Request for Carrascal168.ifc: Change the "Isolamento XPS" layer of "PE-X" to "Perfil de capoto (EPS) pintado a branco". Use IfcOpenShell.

First a look at what the model holds.

```python
import ifcopenshell
import ifcopenshell.util.element

model = ifcopenshell.open("Carrascal168.ifc")
print(model.schema)
for layer_set in model.by_type("IfcMaterialLayerSet"):
    if layer_set.LayerSetName == "PE-X":
        for layer in layer_set.MaterialLayers:
            print(layer.id(), layer.Material and layer.Material.Name, layer.LayerThickness, sep=" | ")
        print(len(ifcopenshell.util.element.get_elements_by_material(model, layer_set)), "elements and types use it")
print(sorted(m.Name for m in model.by_type("IfcMaterial") if m.Name)[:60])
```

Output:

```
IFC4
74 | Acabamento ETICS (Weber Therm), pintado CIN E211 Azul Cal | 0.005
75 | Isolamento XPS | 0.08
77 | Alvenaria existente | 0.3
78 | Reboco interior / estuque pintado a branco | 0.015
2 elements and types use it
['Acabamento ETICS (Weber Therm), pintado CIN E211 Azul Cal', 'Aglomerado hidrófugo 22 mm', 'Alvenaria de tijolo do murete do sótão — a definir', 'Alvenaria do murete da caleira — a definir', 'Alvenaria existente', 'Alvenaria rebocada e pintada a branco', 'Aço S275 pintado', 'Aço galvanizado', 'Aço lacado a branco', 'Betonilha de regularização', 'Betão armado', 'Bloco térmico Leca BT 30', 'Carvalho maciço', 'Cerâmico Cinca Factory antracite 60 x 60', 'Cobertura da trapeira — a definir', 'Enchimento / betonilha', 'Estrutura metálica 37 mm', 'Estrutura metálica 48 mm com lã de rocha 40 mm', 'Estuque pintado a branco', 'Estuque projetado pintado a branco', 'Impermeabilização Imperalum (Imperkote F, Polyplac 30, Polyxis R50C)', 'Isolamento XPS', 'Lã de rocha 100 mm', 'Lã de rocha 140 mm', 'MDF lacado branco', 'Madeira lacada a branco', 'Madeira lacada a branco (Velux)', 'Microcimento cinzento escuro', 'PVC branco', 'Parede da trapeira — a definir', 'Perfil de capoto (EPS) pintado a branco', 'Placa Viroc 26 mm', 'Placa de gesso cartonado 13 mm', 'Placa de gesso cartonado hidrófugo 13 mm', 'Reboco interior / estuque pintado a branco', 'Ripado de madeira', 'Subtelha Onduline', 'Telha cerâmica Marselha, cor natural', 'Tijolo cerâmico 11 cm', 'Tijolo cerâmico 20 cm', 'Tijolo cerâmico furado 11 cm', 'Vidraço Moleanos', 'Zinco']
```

```python
import ifcopenshell
import ifcopenshell.api.material

model = ifcopenshell.open("Carrascal168.ifc")

layer_set = next(s for s in model.by_type("IfcMaterialLayerSet") if s.LayerSetName == "PE-X")
layer = next(l for l in layer_set.MaterialLayers if l.Material and l.Material.Name == "Isolamento XPS")
material = next(m for m in model.by_type("IfcMaterial") if m.Name == "Perfil de capoto (EPS) pintado a branco")

# Point this one layer at the other material; renaming the old one would change it everywhere.
ifcopenshell.api.material.edit_layer(model, layer=layer, attributes={"Name": material.Name}, material=material)

print([l.Material.Name if l.Material else None for l in layer_set.MaterialLayers])

model.write("Carrascal168-out.ifc")
```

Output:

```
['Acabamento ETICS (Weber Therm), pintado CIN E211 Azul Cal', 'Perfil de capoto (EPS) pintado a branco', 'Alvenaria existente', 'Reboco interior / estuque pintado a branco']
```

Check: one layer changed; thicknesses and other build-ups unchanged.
